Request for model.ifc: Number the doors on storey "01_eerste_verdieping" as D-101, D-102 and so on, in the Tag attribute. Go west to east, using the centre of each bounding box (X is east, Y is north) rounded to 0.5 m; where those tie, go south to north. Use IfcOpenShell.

First a look at what the model holds.

```python
import ifcopenshell
import ifcopenshell.util.element
import ifcopenshell.util.placement

model = ifcopenshell.open("model.ifc")
print(model.schema)
storey = next(s for s in model.by_type("IfcBuildingStorey") if s.Name == "01_eerste_verdieping")
doors = [e for e in ifcopenshell.util.element.get_decomposition(storey) if e.is_a("IfcDoor")]
for e in sorted(doors, key=lambda e: e.id()):
    origin = ifcopenshell.util.placement.get_local_placement(e.ObjectPlacement)[:3, 3]
    print(e.id(), e.Tag, e.Name, origin.round(2) + 0.0, sep=" | ")
```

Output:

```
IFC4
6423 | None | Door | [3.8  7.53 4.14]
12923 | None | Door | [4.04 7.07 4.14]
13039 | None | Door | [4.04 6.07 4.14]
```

```python
import ifcopenshell
import ifcopenshell.geom
import ifcopenshell.util.element
import ifcopenshell.util.shape

model = ifcopenshell.open("model.ifc")
settings = ifcopenshell.geom.settings()
settings.set("use-world-coords", True)


def centre(element):
    shape = ifcopenshell.geom.create_shape(settings, element)
    return ifcopenshell.util.shape.get_bbox_centroid(shape.geometry)


storey = next(s for s in model.by_type("IfcBuildingStorey") if s.Name == "01_eerste_verdieping")
doors = [e for e in ifcopenshell.util.element.get_decomposition(storey) if e.is_a("IfcDoor")]

# Insertion points can sit at a corner or the storey origin, so sort by the geometry (in metres).
centres = {e: centre(e) for e in doors}
doors.sort(key=lambda e: (round(centres[e][0] / 0.5), centres[e][1]))

for i, e in enumerate(doors, start=1):
    number = f"D-1{i:02d}"
    e.Tag = number
    print(e.id(), number)

model.write("model_v2.ifc")
```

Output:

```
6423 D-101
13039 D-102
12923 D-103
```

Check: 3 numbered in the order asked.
